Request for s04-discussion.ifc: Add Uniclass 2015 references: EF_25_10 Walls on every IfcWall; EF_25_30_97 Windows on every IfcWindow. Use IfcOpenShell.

First a look at what the model holds.

```python
import ifcopenshell

model = ifcopenshell.open("s04-discussion.ifc")
print(model.schema)
print("classifications:", [c.Name for c in model.by_type("IfcClassification")])
for ifc_class in ("IfcDoor", "IfcRoof", "IfcStair", "IfcWall", "IfcWindow"):
    print(ifc_class, len(model.by_type(ifc_class)))
```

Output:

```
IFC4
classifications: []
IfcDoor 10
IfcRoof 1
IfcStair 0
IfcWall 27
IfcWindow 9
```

```python
import ifcopenshell
import ifcopenshell.api.classification

model = ifcopenshell.open("s04-discussion.ifc")

system = ifcopenshell.api.classification.add_classification(model, classification="Uniclass 2015")

codes = {
    "IfcWall": ("EF_25_10", "Walls"),
    "IfcWindow": ("EF_25_30_97", "Windows"),
}
for ifc_class, (code, name) in codes.items():
    products = model.by_type(ifc_class)
    ifcopenshell.api.classification.add_reference(
        model, products=products, classification=system, identification=code, name=name
    )
    print(code, len(products))

model.write("s04-discussion_updated.ifc")
```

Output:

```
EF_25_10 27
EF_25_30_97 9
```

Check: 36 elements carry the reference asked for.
